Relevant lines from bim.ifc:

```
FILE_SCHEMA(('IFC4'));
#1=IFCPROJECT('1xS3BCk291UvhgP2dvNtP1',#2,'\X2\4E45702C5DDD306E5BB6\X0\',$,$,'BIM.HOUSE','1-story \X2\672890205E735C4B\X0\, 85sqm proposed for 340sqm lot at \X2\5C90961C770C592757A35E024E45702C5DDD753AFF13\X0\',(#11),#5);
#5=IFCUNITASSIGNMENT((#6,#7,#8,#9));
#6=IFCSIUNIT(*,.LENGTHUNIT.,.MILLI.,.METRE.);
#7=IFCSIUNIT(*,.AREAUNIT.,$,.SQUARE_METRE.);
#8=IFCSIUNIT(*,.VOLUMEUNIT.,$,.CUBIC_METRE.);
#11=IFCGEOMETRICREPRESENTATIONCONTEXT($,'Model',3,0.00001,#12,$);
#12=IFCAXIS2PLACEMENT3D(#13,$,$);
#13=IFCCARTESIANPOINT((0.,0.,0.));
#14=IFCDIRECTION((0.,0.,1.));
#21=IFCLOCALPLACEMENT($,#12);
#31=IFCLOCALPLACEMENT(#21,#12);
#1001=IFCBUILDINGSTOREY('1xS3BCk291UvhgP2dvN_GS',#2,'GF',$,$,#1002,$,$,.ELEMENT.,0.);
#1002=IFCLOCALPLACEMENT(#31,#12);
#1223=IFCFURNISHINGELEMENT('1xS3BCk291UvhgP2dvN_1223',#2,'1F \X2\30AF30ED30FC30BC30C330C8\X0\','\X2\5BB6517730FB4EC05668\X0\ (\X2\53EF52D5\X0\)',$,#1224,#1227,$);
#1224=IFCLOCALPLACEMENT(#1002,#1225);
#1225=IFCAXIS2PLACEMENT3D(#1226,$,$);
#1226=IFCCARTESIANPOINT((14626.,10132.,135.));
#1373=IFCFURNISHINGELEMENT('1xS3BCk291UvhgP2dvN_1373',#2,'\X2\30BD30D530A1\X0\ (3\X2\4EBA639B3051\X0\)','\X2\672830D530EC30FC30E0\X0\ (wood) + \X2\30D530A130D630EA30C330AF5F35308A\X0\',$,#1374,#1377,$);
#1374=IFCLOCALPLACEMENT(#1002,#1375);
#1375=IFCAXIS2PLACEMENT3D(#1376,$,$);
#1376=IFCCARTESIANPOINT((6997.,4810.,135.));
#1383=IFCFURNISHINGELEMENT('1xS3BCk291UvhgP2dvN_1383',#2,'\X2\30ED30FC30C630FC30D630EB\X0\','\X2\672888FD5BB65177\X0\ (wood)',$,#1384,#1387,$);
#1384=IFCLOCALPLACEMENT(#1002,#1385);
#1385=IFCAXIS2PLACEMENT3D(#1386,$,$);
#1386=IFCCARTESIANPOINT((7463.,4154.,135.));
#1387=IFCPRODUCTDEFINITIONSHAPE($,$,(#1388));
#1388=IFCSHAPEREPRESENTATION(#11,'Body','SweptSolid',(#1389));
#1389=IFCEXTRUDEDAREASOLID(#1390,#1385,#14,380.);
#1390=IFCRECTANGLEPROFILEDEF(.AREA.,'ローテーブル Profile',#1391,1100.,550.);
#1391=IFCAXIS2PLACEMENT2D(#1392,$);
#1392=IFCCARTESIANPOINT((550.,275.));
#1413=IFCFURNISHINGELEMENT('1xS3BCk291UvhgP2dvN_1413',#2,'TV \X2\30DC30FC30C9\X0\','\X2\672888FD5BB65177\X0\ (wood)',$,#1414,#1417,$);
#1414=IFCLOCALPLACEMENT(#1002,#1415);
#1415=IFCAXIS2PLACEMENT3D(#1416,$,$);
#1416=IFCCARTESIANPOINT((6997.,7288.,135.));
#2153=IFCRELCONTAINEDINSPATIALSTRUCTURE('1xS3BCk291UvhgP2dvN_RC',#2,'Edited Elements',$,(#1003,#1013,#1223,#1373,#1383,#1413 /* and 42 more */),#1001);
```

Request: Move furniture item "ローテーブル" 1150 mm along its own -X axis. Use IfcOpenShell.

```python
import ifcopenshell
import ifcopenshell.api.geometry
import ifcopenshell.util.placement
import ifcopenshell.util.unit

model = ifcopenshell.open("bim.ifc")
unit_scale = ifcopenshell.util.unit.calculate_unit_scale(model)

item = model.by_id(1383)
matrix = ifcopenshell.util.placement.get_local_placement(item.ObjectPlacement)
matrix[:3, 3] -= matrix[:3, 0] * 1.15 / unit_scale
ifcopenshell.api.geometry.edit_object_placement(model, product=item, matrix=matrix, is_si=False)

print(ifcopenshell.util.placement.get_local_placement(item.ObjectPlacement).round(3) + 0.0)

model.write("bim-out.ifc")
```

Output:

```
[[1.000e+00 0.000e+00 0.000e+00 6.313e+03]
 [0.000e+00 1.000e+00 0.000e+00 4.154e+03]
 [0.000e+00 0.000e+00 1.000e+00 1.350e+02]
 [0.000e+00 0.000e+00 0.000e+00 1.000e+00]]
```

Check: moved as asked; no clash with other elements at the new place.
